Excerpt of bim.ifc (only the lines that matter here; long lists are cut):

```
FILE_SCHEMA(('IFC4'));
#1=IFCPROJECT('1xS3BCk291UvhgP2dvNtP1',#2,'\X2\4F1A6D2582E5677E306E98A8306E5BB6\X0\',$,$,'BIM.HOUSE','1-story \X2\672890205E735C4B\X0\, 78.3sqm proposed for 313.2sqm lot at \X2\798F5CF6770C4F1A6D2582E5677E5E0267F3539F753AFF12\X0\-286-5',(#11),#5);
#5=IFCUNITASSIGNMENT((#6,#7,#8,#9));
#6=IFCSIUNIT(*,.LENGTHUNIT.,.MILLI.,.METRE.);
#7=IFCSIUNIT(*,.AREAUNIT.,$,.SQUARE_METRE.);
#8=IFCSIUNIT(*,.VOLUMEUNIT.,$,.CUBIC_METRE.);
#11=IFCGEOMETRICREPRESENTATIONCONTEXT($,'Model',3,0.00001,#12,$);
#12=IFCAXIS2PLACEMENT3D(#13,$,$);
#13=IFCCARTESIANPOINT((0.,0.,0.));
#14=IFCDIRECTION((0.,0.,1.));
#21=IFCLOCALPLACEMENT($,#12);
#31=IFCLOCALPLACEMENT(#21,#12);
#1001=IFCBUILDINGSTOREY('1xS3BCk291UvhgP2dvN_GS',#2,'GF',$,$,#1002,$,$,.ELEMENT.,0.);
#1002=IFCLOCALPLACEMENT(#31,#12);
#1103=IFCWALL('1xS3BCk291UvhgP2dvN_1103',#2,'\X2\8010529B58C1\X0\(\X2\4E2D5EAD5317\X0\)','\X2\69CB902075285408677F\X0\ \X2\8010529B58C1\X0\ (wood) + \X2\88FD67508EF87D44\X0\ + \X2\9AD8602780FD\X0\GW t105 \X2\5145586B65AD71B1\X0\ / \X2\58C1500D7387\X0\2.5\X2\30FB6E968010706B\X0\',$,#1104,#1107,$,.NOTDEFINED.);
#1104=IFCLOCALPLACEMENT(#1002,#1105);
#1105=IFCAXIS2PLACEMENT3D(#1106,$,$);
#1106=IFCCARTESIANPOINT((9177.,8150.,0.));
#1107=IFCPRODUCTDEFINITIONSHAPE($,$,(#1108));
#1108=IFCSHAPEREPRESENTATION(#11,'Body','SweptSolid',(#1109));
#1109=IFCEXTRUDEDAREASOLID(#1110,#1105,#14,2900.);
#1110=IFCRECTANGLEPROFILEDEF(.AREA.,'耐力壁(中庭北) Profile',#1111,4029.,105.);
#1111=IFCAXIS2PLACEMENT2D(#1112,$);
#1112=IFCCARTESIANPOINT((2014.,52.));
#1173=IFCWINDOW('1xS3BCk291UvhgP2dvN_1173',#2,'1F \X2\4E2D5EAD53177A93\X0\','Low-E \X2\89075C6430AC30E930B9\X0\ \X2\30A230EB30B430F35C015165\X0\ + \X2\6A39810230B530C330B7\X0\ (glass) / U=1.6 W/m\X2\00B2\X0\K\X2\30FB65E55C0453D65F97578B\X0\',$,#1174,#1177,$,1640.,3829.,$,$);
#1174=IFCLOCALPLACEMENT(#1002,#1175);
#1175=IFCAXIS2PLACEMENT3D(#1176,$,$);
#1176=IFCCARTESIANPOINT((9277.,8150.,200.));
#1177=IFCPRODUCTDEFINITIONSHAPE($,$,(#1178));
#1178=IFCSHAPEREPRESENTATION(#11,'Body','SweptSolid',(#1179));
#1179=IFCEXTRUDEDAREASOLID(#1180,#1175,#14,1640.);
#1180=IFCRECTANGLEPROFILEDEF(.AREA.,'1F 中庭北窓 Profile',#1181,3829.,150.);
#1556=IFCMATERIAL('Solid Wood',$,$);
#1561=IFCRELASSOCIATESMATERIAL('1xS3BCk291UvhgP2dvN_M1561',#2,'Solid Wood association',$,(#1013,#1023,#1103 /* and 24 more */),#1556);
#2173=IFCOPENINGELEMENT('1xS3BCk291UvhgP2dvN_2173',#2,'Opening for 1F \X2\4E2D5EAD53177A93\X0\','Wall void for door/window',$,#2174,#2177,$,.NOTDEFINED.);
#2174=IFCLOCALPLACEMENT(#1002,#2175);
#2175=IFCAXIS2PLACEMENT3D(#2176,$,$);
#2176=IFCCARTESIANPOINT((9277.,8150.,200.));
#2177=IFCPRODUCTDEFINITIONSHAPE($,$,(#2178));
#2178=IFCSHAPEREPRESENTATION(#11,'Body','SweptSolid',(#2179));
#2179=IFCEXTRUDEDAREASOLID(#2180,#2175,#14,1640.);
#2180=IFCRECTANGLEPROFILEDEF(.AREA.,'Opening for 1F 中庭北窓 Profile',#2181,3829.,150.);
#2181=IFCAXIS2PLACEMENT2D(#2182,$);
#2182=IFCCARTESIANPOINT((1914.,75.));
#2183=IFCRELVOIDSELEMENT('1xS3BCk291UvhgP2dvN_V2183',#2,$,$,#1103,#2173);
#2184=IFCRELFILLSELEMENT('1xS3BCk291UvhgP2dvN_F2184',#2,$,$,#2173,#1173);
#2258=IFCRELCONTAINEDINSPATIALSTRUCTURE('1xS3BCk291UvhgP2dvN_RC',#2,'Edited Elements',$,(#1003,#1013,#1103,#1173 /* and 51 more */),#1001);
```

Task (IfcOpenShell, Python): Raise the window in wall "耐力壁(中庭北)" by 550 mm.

```python
import numpy as np
import ifcopenshell
import ifcopenshell.api.geometry
import ifcopenshell.util.placement
import ifcopenshell.util.unit

model = ifcopenshell.open("bim.ifc")
unit_scale = ifcopenshell.util.unit.calculate_unit_scale(model)

window = model.by_id(1173)
opening = window.FillsVoids[0].RelatingOpeningElement
dz = 550.0

shift = np.array([0.0, 0.0, dz])
# The window is not placed relative to its opening, so move both.
for product in (opening, window):
    matrix = ifcopenshell.util.placement.get_local_placement(product.ObjectPlacement)
    matrix[:3, 3] += shift
    ifcopenshell.api.geometry.edit_object_placement(model, product=product, matrix=matrix, is_si=False)

print(f"moved by {dz * unit_scale:+.3f} m")

model.write("bim_rev.ifc")
```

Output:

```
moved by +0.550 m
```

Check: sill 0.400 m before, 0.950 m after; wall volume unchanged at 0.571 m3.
